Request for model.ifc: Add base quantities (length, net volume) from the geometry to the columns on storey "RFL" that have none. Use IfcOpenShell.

First a look at what the model holds.

```python
import ifcopenshell
import ifcopenshell.util.element
import ifcopenshell.util.unit

model = ifcopenshell.open("model.ifc")
print(model.schema)
for unit_type in ("LENGTHUNIT", "AREAUNIT", "VOLUMEUNIT"):
    print(unit_type, ifcopenshell.util.unit.calculate_unit_scale(model, unit_type))
storey = next(s for s in model.by_type("IfcBuildingStorey") if s.Name == "RFL")
columns = [e for e in ifcopenshell.util.element.get_decomposition(storey) if e.is_a("IfcColumn")]
for e in sorted(columns, key=lambda e: e.id()):
    print(e.id(), e.is_a(), e.Name, list(ifcopenshell.util.element.get_psets(e, qtos_only=True)), sep=" | ")
```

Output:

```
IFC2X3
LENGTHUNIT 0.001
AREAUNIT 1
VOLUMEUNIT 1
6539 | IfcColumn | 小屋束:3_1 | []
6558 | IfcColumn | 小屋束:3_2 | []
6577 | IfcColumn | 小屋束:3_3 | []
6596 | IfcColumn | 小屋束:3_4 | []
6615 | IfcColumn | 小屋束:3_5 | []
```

```python
import ifcopenshell
import ifcopenshell.api.pset
import ifcopenshell.geom
import ifcopenshell.util.element
import ifcopenshell.util.shape
import ifcopenshell.util.unit

model = ifcopenshell.open("model.ifc")
unit_scale = ifcopenshell.util.unit.calculate_unit_scale(model)
volume_scale = ifcopenshell.util.unit.calculate_unit_scale(model, "VOLUMEUNIT")
settings = ifcopenshell.geom.settings()

storey = next(s for s in model.by_type("IfcBuildingStorey") if s.Name == "RFL")
columns = [e for e in ifcopenshell.util.element.get_decomposition(storey) if e.is_a("IfcColumn")]

for e in sorted(columns, key=lambda e: e.id()):
    if ifcopenshell.util.element.get_psets(e, qtos_only=True, should_inherit=False):
        continue
    # Geometry comes back in metres, in the element's own axes.
    shape = ifcopenshell.geom.create_shape(settings, e)
    values = {
        "Length": ifcopenshell.util.shape.get_z(shape.geometry) / unit_scale,
        "NetVolume": ifcopenshell.util.shape.get_volume(shape.geometry) / volume_scale,
    }
    qto = ifcopenshell.api.pset.add_qto(model, product=e, name="BaseQuantities")
    ifcopenshell.api.pset.edit_qto(model, qto=qto, properties=values)
    print(e.id(), {k: round(v, 3) for k, v in values.items()})

model.write("model_updated.ifc")
```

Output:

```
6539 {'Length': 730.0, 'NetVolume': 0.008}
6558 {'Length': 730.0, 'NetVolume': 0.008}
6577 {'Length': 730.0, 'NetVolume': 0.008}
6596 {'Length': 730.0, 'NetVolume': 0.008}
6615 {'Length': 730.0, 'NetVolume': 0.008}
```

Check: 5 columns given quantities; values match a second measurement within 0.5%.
